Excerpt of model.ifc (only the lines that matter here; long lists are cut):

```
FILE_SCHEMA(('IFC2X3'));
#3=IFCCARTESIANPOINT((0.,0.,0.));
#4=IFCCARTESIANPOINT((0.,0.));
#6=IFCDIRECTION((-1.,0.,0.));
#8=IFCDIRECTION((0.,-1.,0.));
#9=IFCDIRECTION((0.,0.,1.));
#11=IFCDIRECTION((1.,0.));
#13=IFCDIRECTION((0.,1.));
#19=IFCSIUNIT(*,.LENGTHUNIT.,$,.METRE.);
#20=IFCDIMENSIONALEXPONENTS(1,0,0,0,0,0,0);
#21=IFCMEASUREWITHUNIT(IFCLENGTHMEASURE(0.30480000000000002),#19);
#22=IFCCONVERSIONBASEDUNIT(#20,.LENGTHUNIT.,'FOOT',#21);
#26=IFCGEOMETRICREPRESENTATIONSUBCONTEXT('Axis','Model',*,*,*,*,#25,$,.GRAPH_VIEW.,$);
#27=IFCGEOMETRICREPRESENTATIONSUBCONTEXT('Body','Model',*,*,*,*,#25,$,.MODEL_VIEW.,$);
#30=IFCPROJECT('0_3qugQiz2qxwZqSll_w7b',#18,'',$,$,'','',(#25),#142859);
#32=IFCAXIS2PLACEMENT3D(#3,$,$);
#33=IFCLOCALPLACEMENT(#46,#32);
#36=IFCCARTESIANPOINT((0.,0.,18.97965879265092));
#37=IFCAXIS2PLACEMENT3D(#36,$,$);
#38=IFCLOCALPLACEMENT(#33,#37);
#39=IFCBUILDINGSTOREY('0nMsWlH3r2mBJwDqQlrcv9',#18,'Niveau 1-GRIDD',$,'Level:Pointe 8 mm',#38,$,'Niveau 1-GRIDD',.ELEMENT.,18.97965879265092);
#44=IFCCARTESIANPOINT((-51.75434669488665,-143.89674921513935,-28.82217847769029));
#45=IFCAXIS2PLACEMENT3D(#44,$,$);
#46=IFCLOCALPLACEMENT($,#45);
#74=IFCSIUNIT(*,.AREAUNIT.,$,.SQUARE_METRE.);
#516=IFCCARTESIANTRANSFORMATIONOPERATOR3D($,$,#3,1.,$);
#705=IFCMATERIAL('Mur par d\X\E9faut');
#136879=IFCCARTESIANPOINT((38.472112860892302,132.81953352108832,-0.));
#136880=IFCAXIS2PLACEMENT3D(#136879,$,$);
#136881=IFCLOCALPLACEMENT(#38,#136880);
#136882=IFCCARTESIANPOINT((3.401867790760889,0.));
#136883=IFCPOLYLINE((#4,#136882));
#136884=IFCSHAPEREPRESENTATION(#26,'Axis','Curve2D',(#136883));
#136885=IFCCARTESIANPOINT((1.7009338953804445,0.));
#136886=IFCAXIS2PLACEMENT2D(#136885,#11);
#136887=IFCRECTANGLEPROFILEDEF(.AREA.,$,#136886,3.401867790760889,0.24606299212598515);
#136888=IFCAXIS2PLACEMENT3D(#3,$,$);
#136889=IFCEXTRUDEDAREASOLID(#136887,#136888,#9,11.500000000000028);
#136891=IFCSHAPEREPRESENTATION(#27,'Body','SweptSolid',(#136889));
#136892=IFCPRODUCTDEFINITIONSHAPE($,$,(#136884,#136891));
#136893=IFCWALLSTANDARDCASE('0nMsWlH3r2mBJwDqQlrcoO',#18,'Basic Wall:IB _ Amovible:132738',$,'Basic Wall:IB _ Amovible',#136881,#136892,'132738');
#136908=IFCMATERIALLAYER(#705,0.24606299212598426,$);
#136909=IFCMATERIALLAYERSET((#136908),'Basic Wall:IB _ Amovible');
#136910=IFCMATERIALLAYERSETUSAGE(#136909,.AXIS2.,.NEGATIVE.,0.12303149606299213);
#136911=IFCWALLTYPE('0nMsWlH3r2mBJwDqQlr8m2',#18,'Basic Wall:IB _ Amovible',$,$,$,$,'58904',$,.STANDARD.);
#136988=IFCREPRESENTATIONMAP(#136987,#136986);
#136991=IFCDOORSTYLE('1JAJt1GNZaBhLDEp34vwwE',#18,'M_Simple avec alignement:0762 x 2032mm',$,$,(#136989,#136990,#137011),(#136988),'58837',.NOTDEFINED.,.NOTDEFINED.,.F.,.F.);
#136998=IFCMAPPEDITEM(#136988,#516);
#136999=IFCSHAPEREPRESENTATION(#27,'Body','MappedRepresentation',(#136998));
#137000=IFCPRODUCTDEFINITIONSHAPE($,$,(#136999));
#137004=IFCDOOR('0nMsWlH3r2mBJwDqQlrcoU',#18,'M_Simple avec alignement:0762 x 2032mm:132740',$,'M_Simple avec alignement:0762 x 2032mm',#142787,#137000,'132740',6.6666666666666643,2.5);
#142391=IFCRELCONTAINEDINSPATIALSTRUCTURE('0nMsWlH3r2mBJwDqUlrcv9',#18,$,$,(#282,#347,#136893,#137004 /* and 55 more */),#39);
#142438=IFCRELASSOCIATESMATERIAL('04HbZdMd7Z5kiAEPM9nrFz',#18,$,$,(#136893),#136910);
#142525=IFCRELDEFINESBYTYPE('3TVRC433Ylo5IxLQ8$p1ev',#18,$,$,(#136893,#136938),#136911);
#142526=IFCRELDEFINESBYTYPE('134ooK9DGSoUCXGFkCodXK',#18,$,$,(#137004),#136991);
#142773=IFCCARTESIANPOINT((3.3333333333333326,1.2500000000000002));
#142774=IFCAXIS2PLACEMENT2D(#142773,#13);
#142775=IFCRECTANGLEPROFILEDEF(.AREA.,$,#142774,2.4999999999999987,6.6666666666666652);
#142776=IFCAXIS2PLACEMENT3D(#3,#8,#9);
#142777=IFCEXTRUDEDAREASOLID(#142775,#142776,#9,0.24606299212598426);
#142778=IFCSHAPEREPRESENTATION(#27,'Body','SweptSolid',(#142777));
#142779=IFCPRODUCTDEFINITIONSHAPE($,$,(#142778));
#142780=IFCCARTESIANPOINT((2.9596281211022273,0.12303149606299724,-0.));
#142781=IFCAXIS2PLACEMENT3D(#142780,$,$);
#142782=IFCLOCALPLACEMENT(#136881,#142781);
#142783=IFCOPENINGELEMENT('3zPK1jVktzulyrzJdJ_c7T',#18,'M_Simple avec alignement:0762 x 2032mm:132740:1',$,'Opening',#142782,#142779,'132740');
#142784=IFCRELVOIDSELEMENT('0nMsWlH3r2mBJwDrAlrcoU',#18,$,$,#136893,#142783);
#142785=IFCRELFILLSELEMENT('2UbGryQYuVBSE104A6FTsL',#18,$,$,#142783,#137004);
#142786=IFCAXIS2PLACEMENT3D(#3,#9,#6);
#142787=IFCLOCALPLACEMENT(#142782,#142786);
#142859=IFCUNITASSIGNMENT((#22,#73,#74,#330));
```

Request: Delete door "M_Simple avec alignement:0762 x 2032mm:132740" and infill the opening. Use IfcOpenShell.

```python
import ifcopenshell
import ifcopenshell.api.feature
import ifcopenshell.api.root
import ifcopenshell.geom
import ifcopenshell.util.shape

model = ifcopenshell.open("model.ifc")
settings = ifcopenshell.geom.settings()


def volume(element):
    """Net volume in cubic metres, openings subtracted."""
    shape = ifcopenshell.geom.create_shape(settings, element)
    return ifcopenshell.util.shape.get_volume(shape.geometry)


door = model.by_id(137004)
opening = door.FillsVoids[0].RelatingOpeningElement
wall = opening.VoidsElements[0].RelatingBuildingElement
before = volume(wall)

ifcopenshell.api.root.remove_product(model, product=door)
ifcopenshell.api.feature.remove_feature(model, feature=opening)

after = volume(wall)

print(f"wall volume {before:.3f} -> {after:.3f} m3")

model.write("model-out.ifc")
```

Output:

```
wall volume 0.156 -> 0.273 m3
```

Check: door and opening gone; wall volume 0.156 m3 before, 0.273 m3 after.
